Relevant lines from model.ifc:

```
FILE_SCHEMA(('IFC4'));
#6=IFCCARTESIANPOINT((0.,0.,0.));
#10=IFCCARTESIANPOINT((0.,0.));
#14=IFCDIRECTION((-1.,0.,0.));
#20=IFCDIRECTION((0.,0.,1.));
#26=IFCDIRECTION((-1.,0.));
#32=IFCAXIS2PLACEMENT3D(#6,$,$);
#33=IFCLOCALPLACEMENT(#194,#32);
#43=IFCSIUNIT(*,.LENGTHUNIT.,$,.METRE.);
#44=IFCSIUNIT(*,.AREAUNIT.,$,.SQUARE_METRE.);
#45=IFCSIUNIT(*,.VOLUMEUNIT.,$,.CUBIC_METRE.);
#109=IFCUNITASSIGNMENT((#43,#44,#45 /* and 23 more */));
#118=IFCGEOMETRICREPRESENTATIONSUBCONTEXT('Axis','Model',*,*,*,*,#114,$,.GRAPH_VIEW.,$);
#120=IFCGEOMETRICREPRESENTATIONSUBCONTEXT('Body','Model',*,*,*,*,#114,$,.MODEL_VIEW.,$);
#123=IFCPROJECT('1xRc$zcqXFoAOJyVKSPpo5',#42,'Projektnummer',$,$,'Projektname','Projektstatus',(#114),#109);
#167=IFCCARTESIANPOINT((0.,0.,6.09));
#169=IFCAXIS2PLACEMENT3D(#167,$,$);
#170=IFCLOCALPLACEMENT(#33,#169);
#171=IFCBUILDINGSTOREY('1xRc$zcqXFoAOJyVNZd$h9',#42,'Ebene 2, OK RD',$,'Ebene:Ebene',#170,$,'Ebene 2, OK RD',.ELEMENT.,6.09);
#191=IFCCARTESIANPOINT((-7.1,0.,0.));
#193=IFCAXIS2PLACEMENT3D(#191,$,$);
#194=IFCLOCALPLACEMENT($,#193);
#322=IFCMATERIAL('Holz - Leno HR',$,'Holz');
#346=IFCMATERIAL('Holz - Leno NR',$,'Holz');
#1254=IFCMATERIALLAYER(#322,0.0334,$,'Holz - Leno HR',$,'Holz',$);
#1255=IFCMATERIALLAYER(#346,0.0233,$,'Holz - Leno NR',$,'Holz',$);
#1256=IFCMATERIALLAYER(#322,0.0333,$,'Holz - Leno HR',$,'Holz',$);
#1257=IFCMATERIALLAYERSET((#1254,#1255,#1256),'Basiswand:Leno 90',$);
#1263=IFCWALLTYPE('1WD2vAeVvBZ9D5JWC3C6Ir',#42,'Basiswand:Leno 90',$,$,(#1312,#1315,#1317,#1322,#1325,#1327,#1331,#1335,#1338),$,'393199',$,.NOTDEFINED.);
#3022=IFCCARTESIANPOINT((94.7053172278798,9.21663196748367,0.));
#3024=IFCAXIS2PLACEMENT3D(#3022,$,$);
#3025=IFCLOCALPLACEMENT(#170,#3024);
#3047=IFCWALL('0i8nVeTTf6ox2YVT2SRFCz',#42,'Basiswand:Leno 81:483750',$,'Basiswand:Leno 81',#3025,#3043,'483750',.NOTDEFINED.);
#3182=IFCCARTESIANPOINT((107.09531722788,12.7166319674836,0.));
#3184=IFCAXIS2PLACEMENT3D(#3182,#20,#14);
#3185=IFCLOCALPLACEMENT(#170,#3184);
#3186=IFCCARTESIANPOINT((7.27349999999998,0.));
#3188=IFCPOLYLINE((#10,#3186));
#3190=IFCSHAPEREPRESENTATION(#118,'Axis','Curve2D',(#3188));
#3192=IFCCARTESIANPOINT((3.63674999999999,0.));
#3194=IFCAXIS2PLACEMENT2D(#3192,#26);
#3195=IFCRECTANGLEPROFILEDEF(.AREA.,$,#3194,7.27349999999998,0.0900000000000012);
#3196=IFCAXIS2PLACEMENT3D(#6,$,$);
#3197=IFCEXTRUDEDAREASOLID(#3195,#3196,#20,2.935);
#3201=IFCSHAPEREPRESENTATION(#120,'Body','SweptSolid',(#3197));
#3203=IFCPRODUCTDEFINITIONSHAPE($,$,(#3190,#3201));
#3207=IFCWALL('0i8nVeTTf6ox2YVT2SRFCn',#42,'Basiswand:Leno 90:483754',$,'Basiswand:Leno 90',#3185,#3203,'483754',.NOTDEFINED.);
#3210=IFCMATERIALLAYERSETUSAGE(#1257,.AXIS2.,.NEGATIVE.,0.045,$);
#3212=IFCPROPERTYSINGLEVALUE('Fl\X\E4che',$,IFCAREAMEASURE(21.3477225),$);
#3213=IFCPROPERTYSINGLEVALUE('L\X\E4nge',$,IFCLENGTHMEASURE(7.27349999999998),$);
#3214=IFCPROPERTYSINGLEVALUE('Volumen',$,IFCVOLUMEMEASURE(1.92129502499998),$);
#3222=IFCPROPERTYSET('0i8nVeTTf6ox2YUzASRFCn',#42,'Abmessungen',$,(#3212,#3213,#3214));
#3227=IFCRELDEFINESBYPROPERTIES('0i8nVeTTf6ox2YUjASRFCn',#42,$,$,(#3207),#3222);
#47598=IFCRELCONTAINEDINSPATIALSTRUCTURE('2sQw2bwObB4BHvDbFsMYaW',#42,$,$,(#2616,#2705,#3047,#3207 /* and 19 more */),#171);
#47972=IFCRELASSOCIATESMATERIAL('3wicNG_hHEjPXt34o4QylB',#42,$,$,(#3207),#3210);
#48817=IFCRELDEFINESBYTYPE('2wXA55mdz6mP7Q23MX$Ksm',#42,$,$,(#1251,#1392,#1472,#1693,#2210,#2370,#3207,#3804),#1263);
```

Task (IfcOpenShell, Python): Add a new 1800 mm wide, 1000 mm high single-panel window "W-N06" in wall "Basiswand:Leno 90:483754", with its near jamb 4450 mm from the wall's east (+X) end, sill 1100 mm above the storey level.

```python
import numpy as np
import ifcopenshell
import ifcopenshell.api.feature
import ifcopenshell.api.geometry
import ifcopenshell.api.pset
import ifcopenshell.api.root
import ifcopenshell.api.spatial
import ifcopenshell.geom
import ifcopenshell.util.element
import ifcopenshell.util.placement
import ifcopenshell.util.representation
import ifcopenshell.util.shape
import ifcopenshell.util.unit

model = ifcopenshell.open("model.ifc")
unit_scale = ifcopenshell.util.unit.calculate_unit_scale(model)
area_scale = ifcopenshell.util.unit.calculate_unit_scale(model, "AREAUNIT")
volume_scale = ifcopenshell.util.unit.calculate_unit_scale(model, "VOLUMEUNIT")
settings = ifcopenshell.geom.settings()


def volume(element):
    """Net volume in cubic metres, openings subtracted."""
    shape = ifcopenshell.geom.create_shape(settings, element)
    return ifcopenshell.util.shape.get_volume(shape.geometry)


wall = model.by_guid("0i8nVeTTf6ox2YVT2SRFCn")
storey = ifcopenshell.util.element.get_container(wall, ifc_class="IfcBuildingStorey")
context = ifcopenshell.util.representation.get_context(model, "Model", "Body", "MODEL_VIEW")
before = volume(wall)

width, height, from_end, sill = 1.8, 1, 4.45, 1.1  # metres

# The wall runs along its own X axis, and the end named is its -X end.
wall_shape = ifcopenshell.geom.create_shape(settings, wall)
x, y, z = ifcopenshell.util.shape.get_vertices(wall_shape.geometry).T
start = x.min() + from_end
face, thickness = float(y.min()), float(y.max() - y.min())
wall_matrix = ifcopenshell.util.placement.get_local_placement(wall.ObjectPlacement)
level = ifcopenshell.util.placement.get_local_placement(storey.ObjectPlacement)[2, 3]


def in_wall(x, y):
    """Placement at x, y metres in the wall's axes, at sill height."""
    matrix = wall_matrix.copy()
    matrix[:, 3] = wall_matrix @ np.array([x / unit_scale, y / unit_scale, 0.0, 1.0])
    matrix[2, 3] = level + sill / unit_scale
    return matrix


# Opening: a box that overshoots both wall faces by 50 mm.
opening = ifcopenshell.api.root.create_entity(model, ifc_class="IfcOpeningElement", predefined_type="OPENING")
box = ifcopenshell.api.geometry.add_wall_representation(
    model, context=context, length=width, height=height, thickness=thickness + 0.1
)
ifcopenshell.api.geometry.assign_representation(model, product=opening, representation=box)
ifcopenshell.api.geometry.edit_object_placement(model, product=opening, matrix=in_wall(start, face - 0.05), is_si=False)
ifcopenshell.api.feature.add_feature(model, feature=opening, element=wall)

window = ifcopenshell.api.root.create_entity(model, ifc_class="IfcWindow", name="W-N06", predefined_type="WINDOW")
window.OverallWidth, window.OverallHeight = width / unit_scale, height / unit_scale
window.PartitioningType = "SINGLE_PANEL"
body = ifcopenshell.api.geometry.add_window_representation(
    model,
    context=context,
    overall_width=window.OverallWidth,
    overall_height=window.OverallHeight,
    partition_type="SINGLE_PANEL",
)
ifcopenshell.api.geometry.assign_representation(model, product=window, representation=body)
ifcopenshell.api.spatial.assign_container(model, products=[window], relating_structure=storey)
ifcopenshell.api.feature.add_filling(model, opening=opening, element=window)

# Centre the window in the wall's thickness.
ifcopenshell.api.geometry.edit_object_placement(model, product=window, matrix=in_wall(start, face), is_si=False)
window_shape = ifcopenshell.geom.create_shape(settings, window)
depth = ifcopenshell.util.shape.get_vertices(window_shape.geometry)[:, 1]
offset = face + thickness / 2 - (depth.min() + depth.max()) / 2
ifcopenshell.api.geometry.edit_object_placement(model, product=window, matrix=in_wall(start, offset), is_si=False)

after = volume(wall)

# Update the wall's stored quantities.
pset = model.by_id(ifcopenshell.util.element.get_pset(wall, "Abmessungen", should_inherit=False)["id"])
ifcopenshell.api.pset.edit_pset(model, pset=pset, properties={
    "Fläche": model.create_entity("IfcAreaMeasure", after / thickness / area_scale),
    "Volumen": model.create_entity("IfcVolumeMeasure", after / volume_scale),
})

print(f"wall volume {before:.3f} -> {after:.3f} m3")

model.write("model_updated.ifc")
```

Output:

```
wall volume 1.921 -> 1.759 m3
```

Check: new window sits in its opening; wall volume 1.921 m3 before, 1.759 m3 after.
